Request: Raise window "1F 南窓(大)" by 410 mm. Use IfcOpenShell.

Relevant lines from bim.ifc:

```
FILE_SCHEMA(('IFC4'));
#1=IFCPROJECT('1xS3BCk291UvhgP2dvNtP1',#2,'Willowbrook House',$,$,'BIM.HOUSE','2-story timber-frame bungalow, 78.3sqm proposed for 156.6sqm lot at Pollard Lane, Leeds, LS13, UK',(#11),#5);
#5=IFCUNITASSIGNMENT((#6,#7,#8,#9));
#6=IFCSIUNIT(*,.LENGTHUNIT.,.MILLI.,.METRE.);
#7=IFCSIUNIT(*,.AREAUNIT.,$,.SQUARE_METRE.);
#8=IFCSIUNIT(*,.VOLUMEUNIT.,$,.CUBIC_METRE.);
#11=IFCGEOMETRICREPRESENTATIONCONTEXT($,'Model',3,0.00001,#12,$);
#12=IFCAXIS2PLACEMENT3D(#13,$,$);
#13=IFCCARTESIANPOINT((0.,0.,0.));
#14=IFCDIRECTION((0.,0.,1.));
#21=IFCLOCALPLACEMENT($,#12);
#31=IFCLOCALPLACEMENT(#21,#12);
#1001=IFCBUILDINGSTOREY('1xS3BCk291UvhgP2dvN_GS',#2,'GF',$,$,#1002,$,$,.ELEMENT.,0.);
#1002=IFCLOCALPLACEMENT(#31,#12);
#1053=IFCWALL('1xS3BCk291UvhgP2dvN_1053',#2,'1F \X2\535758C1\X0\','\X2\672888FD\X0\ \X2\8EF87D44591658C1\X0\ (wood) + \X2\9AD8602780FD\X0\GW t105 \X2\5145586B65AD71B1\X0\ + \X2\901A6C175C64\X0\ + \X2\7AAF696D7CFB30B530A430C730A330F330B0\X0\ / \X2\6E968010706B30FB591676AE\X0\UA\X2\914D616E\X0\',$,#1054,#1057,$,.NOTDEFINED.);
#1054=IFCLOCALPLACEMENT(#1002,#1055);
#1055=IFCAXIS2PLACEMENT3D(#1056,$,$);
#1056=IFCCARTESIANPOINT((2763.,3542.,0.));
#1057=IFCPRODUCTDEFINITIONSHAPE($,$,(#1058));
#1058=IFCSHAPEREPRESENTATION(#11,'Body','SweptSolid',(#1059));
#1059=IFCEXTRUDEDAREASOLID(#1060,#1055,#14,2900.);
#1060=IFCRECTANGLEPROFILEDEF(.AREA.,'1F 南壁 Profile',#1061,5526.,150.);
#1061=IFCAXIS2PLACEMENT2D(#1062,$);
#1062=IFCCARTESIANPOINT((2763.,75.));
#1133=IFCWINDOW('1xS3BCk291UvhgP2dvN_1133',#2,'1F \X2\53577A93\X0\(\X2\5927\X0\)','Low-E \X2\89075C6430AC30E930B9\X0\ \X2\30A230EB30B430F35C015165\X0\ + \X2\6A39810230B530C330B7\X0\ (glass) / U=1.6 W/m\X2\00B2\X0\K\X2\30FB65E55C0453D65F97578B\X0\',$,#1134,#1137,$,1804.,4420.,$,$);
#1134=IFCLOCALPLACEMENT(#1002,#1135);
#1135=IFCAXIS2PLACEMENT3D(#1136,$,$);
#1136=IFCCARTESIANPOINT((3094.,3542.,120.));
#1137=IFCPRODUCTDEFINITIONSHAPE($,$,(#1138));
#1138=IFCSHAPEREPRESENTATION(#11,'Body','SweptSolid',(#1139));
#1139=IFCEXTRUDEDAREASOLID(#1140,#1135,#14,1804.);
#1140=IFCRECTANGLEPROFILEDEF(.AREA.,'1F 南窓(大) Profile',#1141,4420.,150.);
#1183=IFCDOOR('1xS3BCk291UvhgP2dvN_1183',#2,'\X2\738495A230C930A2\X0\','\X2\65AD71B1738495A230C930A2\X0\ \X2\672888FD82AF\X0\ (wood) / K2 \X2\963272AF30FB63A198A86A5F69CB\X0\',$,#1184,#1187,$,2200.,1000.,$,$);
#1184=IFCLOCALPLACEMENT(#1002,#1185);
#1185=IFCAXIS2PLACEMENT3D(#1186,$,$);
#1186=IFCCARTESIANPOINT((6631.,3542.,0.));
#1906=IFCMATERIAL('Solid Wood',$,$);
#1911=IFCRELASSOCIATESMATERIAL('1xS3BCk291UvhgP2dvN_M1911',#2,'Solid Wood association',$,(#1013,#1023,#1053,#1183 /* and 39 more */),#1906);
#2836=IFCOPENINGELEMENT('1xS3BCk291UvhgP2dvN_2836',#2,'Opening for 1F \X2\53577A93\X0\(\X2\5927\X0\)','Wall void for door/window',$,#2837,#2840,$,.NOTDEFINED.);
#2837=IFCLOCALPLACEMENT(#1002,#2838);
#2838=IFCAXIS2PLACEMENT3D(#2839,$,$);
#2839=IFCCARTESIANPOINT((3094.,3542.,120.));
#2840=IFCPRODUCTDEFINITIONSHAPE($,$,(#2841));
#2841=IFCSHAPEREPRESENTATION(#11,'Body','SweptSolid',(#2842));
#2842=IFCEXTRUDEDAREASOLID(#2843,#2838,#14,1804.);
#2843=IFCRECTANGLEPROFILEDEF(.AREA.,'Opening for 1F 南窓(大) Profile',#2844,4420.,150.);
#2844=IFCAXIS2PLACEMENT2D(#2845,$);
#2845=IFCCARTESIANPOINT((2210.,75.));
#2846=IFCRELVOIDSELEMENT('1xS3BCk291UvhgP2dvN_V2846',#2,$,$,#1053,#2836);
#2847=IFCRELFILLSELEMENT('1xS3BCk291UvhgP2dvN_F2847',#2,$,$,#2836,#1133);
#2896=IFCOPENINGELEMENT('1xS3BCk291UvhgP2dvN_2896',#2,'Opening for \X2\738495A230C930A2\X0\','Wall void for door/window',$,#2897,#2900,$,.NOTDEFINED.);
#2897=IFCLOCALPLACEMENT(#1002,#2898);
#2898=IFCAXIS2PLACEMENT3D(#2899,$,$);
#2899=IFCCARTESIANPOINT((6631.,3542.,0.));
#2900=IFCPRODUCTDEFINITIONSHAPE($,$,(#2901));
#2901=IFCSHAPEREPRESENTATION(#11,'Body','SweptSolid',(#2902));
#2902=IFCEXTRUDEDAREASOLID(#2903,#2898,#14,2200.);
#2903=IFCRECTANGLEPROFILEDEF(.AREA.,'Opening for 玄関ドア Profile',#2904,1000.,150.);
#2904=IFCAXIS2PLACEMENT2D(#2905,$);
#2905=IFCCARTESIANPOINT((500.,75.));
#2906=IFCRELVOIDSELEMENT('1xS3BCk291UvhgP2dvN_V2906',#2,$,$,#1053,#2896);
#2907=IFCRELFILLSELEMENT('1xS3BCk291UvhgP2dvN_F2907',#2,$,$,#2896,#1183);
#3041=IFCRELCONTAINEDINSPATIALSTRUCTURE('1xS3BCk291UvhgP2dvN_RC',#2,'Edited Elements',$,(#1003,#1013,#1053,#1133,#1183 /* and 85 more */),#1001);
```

```python
import numpy as np
import ifcopenshell
import ifcopenshell.api.geometry
import ifcopenshell.util.placement
import ifcopenshell.util.unit

model = ifcopenshell.open("bim.ifc")
unit_scale = ifcopenshell.util.unit.calculate_unit_scale(model)

window = model.by_guid("1xS3BCk291UvhgP2dvN_1133")
opening = window.FillsVoids[0].RelatingOpeningElement
dz = 0.41 / unit_scale

shift = np.array([0.0, 0.0, dz])
# The window is not placed relative to its opening, so move both.
for product in (opening, window):
    matrix = ifcopenshell.util.placement.get_local_placement(product.ObjectPlacement)
    matrix[:3, 3] += shift
    ifcopenshell.api.geometry.edit_object_placement(model, product=product, matrix=matrix, is_si=False)

print(f"moved by {dz * unit_scale:+.3f} m")

model.write("bim_rev.ifc")
```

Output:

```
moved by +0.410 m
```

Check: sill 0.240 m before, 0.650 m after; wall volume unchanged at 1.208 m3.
